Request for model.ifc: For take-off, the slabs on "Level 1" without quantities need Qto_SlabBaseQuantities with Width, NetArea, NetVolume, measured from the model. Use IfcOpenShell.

First a look at what the model holds.

```python
import ifcopenshell
import ifcopenshell.util.element
import ifcopenshell.util.unit

model = ifcopenshell.open("model.ifc")
print(model.schema)
for unit_type in ("LENGTHUNIT", "AREAUNIT", "VOLUMEUNIT"):
    print(unit_type, ifcopenshell.util.unit.calculate_unit_scale(model, unit_type))
storey = next(s for s in model.by_type("IfcBuildingStorey") if s.Name == "Level 1")
slabs = [e for e in ifcopenshell.util.element.get_decomposition(storey) if e.is_a("IfcSlab")]
for e in sorted(slabs, key=lambda e: e.id()):
    print(e.id(), e.is_a(), e.Name, list(ifcopenshell.util.element.get_psets(e, qtos_only=True)), sep=" | ")
```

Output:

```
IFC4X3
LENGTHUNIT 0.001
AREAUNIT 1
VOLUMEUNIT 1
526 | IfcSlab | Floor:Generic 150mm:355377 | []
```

```python
import ifcopenshell
import ifcopenshell.api.pset
import ifcopenshell.geom
import ifcopenshell.util.element
import ifcopenshell.util.shape
import ifcopenshell.util.unit

model = ifcopenshell.open("model.ifc")
unit_scale = ifcopenshell.util.unit.calculate_unit_scale(model)
area_scale = ifcopenshell.util.unit.calculate_unit_scale(model, "AREAUNIT")
volume_scale = ifcopenshell.util.unit.calculate_unit_scale(model, "VOLUMEUNIT")
settings = ifcopenshell.geom.settings()

storey = next(s for s in model.by_type("IfcBuildingStorey") if s.Name == "Level 1")
slabs = [e for e in ifcopenshell.util.element.get_decomposition(storey) if e.is_a("IfcSlab")]

for e in sorted(slabs, key=lambda e: e.id()):
    if ifcopenshell.util.element.get_psets(e, qtos_only=True, should_inherit=False):
        continue
    # Geometry comes back in metres, in the element's own axes.
    shape = ifcopenshell.geom.create_shape(settings, e)
    values = {
        "Width": ifcopenshell.util.shape.get_z(shape.geometry) / unit_scale,
        "NetArea": ifcopenshell.util.shape.get_footprint_area(shape.geometry) / area_scale,
        "NetVolume": ifcopenshell.util.shape.get_volume(shape.geometry) / volume_scale,
    }
    qto = ifcopenshell.api.pset.add_qto(model, product=e, name="Qto_SlabBaseQuantities")
    ifcopenshell.api.pset.edit_qto(model, qto=qto, properties=values)
    print(e.id(), {k: round(v, 3) for k, v in values.items()})

model.write("model_v2.ifc")
```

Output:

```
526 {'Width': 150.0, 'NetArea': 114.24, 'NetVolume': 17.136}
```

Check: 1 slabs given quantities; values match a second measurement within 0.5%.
